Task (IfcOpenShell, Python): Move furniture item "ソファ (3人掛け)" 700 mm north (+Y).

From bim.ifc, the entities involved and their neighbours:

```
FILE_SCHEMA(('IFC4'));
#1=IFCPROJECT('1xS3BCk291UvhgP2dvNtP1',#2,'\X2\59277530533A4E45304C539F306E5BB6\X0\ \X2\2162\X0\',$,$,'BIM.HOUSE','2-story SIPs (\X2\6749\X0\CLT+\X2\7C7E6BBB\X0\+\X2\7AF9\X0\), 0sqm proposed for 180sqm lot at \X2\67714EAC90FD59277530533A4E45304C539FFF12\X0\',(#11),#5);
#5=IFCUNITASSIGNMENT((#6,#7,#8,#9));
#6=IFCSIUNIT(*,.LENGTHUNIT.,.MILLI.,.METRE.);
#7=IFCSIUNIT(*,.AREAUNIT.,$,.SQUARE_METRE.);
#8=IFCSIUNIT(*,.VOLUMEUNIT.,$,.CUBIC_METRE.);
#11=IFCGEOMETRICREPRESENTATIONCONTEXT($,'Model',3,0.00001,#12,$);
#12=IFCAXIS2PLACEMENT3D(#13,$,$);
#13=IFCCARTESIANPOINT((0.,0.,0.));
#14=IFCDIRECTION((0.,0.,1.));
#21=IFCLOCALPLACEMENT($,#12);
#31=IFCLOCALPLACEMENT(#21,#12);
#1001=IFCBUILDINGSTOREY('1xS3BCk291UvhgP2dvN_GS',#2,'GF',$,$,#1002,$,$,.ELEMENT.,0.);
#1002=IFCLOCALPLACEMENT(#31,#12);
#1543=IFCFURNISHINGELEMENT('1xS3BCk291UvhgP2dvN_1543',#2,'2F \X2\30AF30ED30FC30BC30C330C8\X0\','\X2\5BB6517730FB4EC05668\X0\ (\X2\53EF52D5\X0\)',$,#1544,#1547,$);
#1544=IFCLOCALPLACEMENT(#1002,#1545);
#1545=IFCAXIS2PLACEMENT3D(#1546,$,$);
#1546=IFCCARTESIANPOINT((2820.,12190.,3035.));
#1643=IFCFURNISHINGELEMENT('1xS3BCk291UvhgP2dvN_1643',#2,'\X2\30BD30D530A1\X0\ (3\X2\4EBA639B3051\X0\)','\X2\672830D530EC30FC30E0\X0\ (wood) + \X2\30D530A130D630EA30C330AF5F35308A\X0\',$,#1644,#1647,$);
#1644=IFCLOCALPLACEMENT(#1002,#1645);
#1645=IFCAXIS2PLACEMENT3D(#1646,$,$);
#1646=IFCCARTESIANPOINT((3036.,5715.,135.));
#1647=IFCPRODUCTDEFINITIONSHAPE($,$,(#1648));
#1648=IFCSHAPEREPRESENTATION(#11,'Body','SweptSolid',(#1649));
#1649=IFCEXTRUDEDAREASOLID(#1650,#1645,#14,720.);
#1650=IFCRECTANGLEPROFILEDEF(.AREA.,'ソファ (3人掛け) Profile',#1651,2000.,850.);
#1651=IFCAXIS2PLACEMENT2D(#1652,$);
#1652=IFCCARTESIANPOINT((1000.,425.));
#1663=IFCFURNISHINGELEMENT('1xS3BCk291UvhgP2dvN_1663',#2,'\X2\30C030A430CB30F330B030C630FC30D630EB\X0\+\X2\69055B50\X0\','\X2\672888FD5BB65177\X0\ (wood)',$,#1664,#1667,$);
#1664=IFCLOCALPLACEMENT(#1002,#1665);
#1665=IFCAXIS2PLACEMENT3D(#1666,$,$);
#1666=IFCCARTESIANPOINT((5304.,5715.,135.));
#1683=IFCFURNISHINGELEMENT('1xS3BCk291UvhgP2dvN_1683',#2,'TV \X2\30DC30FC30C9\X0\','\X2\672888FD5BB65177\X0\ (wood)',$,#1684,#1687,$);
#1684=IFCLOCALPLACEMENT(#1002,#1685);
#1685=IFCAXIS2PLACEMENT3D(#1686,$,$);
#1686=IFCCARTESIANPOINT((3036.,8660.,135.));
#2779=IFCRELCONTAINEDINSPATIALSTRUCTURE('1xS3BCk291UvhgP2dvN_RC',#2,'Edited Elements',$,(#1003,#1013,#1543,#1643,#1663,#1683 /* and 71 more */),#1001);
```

```python
import ifcopenshell
import ifcopenshell.api.geometry
import ifcopenshell.util.placement
import ifcopenshell.util.unit

model = ifcopenshell.open("bim.ifc")
unit_scale = ifcopenshell.util.unit.calculate_unit_scale(model)

item = model.by_guid("1xS3BCk291UvhgP2dvN_1643")
matrix = ifcopenshell.util.placement.get_local_placement(item.ObjectPlacement)
matrix[1, 3] += 0.7 / unit_scale
ifcopenshell.api.geometry.edit_object_placement(model, product=item, matrix=matrix, is_si=False)

print(ifcopenshell.util.placement.get_local_placement(item.ObjectPlacement).round(3) + 0.0)

model.write("bim_updated.ifc")
```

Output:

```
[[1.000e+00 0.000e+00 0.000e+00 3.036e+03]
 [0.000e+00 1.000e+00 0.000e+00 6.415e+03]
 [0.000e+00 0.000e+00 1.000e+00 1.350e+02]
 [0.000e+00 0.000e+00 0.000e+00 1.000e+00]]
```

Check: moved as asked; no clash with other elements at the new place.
